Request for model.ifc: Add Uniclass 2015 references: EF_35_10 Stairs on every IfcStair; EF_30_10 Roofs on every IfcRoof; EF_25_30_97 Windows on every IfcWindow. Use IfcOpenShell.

First a look at what the model holds.

```python
import ifcopenshell

model = ifcopenshell.open("model.ifc")
print(model.schema)
print("classifications:", [c.Name for c in model.by_type("IfcClassification")])
for ifc_class in ("IfcDoor", "IfcRoof", "IfcStair", "IfcWall", "IfcWindow"):
    print(ifc_class, len(model.by_type(ifc_class)))
```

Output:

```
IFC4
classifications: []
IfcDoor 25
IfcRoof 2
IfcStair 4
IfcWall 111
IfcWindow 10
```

```python
import ifcopenshell
import ifcopenshell.api.classification

model = ifcopenshell.open("model.ifc")

system = ifcopenshell.api.classification.add_classification(model, classification="Uniclass 2015")

codes = {
    "IfcStair": ("EF_35_10", "Stairs"),
    "IfcRoof": ("EF_30_10", "Roofs"),
    "IfcWindow": ("EF_25_30_97", "Windows"),
}
for ifc_class, (code, name) in codes.items():
    products = model.by_type(ifc_class)
    ifcopenshell.api.classification.add_reference(
        model, products=products, classification=system, identification=code, name=name
    )
    print(code, len(products))

model.write("model_rev.ifc")
```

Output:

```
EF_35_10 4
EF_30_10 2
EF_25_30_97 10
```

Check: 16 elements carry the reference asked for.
